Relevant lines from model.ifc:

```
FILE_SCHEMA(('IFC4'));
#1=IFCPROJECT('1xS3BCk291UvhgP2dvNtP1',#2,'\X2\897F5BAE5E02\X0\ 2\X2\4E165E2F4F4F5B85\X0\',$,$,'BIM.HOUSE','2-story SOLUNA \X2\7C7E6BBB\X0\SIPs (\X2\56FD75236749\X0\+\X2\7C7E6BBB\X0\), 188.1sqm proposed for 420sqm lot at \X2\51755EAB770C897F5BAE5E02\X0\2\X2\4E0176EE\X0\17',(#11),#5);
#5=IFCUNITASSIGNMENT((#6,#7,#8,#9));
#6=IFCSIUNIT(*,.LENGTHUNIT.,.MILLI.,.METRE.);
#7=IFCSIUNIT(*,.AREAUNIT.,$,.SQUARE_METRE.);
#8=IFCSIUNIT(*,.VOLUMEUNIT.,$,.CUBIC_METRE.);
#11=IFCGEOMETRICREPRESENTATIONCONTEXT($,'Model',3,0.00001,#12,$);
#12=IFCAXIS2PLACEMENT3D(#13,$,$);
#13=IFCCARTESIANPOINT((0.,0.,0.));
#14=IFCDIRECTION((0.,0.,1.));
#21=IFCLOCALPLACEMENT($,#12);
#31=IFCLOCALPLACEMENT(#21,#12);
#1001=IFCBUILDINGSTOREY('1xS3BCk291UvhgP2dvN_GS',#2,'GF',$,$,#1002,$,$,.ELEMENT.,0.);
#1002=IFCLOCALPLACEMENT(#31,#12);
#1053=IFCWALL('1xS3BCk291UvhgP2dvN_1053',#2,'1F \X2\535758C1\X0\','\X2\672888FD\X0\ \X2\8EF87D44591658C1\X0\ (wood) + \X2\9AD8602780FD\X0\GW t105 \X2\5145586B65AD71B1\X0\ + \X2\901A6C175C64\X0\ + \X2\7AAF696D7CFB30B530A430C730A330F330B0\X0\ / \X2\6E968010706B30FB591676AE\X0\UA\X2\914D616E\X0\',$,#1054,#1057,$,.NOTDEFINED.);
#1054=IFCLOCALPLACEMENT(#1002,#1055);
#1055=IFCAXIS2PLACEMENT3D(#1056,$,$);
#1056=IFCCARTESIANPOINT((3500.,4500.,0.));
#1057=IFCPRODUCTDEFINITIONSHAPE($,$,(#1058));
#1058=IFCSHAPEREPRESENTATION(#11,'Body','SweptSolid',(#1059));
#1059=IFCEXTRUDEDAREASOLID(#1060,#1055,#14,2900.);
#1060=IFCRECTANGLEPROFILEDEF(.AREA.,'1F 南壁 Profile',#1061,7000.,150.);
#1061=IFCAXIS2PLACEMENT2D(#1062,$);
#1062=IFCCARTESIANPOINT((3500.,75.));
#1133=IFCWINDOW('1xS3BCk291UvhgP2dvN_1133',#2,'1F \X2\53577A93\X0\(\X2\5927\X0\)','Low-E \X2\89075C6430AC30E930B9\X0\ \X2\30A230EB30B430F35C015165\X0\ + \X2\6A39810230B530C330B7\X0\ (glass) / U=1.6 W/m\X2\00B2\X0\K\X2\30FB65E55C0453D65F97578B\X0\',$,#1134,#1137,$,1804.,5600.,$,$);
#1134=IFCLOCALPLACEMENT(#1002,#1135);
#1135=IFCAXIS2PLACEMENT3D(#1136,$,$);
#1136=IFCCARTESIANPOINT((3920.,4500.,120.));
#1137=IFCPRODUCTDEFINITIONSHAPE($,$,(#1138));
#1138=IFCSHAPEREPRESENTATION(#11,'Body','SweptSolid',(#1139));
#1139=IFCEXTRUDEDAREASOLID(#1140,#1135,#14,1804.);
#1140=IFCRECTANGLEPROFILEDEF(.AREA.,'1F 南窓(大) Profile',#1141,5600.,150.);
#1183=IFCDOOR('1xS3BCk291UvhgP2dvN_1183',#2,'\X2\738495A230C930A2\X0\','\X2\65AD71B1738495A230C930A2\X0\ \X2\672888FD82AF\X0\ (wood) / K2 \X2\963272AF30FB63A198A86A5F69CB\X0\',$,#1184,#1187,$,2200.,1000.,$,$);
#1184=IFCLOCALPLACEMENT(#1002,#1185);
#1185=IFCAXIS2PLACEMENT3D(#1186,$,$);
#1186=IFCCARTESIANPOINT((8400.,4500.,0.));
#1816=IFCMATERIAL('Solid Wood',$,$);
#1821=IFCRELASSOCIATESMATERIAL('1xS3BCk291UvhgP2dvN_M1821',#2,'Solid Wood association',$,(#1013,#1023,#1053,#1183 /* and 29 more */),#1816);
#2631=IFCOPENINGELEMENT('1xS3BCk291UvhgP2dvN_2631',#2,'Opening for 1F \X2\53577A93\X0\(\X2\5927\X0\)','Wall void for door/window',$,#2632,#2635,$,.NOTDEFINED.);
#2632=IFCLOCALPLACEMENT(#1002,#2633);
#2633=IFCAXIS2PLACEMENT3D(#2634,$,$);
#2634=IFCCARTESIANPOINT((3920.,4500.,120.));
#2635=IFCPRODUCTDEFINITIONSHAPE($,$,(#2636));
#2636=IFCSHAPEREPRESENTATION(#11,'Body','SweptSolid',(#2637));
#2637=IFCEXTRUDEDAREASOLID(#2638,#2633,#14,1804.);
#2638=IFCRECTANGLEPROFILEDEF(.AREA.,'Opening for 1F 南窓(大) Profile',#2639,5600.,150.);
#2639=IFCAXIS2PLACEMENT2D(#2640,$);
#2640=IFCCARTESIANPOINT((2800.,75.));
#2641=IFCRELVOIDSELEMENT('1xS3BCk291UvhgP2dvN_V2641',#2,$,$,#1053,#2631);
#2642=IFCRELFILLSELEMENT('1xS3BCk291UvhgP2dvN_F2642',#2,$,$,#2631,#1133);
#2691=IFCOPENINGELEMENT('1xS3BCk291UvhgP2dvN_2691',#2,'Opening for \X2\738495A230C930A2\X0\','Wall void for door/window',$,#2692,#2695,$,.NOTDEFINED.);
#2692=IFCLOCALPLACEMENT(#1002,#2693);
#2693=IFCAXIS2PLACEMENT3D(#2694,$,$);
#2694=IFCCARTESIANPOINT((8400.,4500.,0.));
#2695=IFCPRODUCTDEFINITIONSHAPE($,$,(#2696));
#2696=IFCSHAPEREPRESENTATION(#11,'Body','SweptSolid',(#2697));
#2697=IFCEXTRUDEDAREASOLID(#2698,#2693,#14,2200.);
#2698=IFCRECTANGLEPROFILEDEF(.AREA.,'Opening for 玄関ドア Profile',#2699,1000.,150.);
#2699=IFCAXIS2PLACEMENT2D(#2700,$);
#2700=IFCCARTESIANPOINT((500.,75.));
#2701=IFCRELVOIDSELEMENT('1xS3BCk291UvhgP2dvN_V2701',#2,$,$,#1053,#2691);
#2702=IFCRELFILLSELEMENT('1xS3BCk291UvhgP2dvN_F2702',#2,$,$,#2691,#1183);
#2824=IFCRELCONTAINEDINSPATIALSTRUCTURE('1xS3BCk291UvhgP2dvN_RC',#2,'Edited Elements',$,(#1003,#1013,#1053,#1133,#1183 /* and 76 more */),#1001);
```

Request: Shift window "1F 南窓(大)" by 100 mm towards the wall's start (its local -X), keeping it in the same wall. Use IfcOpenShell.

```python
import ifcopenshell
import ifcopenshell.api.geometry
import ifcopenshell.util.placement
import ifcopenshell.util.unit

model = ifcopenshell.open("model.ifc")
unit_scale = ifcopenshell.util.unit.calculate_unit_scale(model)

window = model.by_id(1133)
opening = window.FillsVoids[0].RelatingOpeningElement
wall = opening.VoidsElements[0].RelatingBuildingElement

wall_matrix = ifcopenshell.util.placement.get_local_placement(wall.ObjectPlacement)
shift = wall_matrix[:3, 0] * -0.1 / unit_scale
before = ifcopenshell.util.placement.get_local_placement(window.ObjectPlacement)[:3, 3].copy()

# The window is not placed relative to its opening, so move both.
for product in (opening, window):
    matrix = ifcopenshell.util.placement.get_local_placement(product.ObjectPlacement)
    matrix[:3, 3] += shift
    ifcopenshell.api.geometry.edit_object_placement(model, product=product, matrix=matrix, is_si=False)

after = ifcopenshell.util.placement.get_local_placement(window.ObjectPlacement)[:3, 3]
print("window moved by", (after - before).round(3) + 0.0)

model.write("model_rev.ifc")
```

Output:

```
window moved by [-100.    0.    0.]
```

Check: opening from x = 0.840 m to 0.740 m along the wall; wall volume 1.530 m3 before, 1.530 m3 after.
